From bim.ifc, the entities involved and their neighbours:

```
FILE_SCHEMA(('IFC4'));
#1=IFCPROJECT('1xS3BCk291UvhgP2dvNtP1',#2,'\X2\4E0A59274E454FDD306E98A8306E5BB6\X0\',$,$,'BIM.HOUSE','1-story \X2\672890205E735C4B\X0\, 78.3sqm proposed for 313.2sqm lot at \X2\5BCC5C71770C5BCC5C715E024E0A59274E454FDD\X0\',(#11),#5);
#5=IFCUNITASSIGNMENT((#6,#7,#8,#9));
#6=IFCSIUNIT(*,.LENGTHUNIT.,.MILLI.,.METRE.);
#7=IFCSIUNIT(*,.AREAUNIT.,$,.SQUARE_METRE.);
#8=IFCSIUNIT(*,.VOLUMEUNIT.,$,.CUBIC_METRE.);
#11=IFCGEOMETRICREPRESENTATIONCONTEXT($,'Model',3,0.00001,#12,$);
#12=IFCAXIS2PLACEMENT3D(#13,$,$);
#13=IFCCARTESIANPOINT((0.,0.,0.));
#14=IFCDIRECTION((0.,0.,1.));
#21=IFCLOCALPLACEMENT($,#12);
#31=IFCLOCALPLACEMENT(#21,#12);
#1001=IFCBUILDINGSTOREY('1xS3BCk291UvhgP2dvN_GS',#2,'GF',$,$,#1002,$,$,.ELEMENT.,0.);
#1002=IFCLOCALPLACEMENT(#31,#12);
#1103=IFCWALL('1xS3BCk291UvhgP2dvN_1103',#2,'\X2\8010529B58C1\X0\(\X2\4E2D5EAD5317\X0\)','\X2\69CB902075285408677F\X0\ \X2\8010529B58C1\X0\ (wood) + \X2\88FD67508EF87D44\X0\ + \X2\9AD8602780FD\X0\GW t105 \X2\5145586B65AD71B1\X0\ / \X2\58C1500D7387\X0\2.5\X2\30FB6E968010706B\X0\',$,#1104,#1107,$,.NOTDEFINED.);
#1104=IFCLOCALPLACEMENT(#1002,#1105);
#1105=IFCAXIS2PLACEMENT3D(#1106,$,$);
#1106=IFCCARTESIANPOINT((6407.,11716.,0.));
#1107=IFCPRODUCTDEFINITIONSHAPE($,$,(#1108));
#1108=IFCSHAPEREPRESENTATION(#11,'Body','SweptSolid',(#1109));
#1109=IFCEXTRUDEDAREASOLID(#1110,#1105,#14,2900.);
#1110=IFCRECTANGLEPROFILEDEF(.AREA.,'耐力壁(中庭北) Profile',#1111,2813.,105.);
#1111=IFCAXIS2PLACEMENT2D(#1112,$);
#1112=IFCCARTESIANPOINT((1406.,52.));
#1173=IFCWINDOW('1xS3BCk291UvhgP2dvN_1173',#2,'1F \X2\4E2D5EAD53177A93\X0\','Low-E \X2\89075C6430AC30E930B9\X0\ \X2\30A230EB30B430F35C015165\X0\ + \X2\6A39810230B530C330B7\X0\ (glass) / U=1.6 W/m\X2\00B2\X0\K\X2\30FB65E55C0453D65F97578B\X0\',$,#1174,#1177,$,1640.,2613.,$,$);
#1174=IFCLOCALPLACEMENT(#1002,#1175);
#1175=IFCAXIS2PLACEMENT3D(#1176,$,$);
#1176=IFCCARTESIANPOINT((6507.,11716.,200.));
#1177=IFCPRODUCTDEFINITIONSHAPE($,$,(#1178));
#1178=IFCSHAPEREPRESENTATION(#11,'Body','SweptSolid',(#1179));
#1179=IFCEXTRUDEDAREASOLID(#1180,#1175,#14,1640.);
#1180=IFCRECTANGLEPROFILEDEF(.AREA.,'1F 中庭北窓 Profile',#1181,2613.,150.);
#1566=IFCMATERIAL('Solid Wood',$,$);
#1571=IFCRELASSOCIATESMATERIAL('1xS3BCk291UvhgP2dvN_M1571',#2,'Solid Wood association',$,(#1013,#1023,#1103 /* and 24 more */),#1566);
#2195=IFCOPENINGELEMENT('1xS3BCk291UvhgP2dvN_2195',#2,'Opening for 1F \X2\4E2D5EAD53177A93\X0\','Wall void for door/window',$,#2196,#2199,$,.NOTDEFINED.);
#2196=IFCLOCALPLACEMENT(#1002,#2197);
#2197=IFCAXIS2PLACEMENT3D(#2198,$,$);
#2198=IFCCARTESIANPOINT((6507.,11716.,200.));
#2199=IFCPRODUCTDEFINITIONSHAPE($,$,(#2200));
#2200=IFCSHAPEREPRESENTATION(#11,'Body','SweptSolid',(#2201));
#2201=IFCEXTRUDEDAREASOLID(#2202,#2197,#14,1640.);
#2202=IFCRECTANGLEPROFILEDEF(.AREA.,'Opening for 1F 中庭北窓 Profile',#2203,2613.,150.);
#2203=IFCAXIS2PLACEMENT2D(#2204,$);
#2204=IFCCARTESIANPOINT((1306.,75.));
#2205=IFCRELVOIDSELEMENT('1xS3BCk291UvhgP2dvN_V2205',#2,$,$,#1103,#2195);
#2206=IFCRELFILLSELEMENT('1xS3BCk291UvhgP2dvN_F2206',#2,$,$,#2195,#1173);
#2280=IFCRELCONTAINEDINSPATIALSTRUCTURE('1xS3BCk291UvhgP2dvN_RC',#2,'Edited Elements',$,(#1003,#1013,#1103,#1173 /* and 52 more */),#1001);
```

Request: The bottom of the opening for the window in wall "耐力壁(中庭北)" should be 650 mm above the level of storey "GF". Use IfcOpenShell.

```python
import numpy as np
import ifcopenshell
import ifcopenshell.api.geometry
import ifcopenshell.geom
import ifcopenshell.util.element
import ifcopenshell.util.placement
import ifcopenshell.util.shape
import ifcopenshell.util.unit

model = ifcopenshell.open("bim.ifc")
unit_scale = ifcopenshell.util.unit.calculate_unit_scale(model)

window = model.by_guid("1xS3BCk291UvhgP2dvN_1173")
opening = window.FillsVoids[0].RelatingOpeningElement
storey = ifcopenshell.util.element.get_container(window, ifc_class="IfcBuildingStorey")
level = ifcopenshell.util.placement.get_local_placement(storey.ObjectPlacement)[2, 3]

# The opening's origin need not be at the sill, so measure its lowest point.
shape = ifcopenshell.geom.create_shape(ifcopenshell.geom.settings(), opening)
bottom = ifcopenshell.util.shape.get_shape_bottom_elevation(shape, shape.geometry) / unit_scale
dz = level + 0.65 / unit_scale - bottom

shift = np.array([0.0, 0.0, dz])
# The window is not placed relative to its opening, so move both.
for product in (opening, window):
    matrix = ifcopenshell.util.placement.get_local_placement(product.ObjectPlacement)
    matrix[:3, 3] += shift
    ifcopenshell.api.geometry.edit_object_placement(model, product=product, matrix=matrix, is_si=False)

print(f"moved by {dz * unit_scale:+.3f} m")

model.write("bim-out.ifc")
```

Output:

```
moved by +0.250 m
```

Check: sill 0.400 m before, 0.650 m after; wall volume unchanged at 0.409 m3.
